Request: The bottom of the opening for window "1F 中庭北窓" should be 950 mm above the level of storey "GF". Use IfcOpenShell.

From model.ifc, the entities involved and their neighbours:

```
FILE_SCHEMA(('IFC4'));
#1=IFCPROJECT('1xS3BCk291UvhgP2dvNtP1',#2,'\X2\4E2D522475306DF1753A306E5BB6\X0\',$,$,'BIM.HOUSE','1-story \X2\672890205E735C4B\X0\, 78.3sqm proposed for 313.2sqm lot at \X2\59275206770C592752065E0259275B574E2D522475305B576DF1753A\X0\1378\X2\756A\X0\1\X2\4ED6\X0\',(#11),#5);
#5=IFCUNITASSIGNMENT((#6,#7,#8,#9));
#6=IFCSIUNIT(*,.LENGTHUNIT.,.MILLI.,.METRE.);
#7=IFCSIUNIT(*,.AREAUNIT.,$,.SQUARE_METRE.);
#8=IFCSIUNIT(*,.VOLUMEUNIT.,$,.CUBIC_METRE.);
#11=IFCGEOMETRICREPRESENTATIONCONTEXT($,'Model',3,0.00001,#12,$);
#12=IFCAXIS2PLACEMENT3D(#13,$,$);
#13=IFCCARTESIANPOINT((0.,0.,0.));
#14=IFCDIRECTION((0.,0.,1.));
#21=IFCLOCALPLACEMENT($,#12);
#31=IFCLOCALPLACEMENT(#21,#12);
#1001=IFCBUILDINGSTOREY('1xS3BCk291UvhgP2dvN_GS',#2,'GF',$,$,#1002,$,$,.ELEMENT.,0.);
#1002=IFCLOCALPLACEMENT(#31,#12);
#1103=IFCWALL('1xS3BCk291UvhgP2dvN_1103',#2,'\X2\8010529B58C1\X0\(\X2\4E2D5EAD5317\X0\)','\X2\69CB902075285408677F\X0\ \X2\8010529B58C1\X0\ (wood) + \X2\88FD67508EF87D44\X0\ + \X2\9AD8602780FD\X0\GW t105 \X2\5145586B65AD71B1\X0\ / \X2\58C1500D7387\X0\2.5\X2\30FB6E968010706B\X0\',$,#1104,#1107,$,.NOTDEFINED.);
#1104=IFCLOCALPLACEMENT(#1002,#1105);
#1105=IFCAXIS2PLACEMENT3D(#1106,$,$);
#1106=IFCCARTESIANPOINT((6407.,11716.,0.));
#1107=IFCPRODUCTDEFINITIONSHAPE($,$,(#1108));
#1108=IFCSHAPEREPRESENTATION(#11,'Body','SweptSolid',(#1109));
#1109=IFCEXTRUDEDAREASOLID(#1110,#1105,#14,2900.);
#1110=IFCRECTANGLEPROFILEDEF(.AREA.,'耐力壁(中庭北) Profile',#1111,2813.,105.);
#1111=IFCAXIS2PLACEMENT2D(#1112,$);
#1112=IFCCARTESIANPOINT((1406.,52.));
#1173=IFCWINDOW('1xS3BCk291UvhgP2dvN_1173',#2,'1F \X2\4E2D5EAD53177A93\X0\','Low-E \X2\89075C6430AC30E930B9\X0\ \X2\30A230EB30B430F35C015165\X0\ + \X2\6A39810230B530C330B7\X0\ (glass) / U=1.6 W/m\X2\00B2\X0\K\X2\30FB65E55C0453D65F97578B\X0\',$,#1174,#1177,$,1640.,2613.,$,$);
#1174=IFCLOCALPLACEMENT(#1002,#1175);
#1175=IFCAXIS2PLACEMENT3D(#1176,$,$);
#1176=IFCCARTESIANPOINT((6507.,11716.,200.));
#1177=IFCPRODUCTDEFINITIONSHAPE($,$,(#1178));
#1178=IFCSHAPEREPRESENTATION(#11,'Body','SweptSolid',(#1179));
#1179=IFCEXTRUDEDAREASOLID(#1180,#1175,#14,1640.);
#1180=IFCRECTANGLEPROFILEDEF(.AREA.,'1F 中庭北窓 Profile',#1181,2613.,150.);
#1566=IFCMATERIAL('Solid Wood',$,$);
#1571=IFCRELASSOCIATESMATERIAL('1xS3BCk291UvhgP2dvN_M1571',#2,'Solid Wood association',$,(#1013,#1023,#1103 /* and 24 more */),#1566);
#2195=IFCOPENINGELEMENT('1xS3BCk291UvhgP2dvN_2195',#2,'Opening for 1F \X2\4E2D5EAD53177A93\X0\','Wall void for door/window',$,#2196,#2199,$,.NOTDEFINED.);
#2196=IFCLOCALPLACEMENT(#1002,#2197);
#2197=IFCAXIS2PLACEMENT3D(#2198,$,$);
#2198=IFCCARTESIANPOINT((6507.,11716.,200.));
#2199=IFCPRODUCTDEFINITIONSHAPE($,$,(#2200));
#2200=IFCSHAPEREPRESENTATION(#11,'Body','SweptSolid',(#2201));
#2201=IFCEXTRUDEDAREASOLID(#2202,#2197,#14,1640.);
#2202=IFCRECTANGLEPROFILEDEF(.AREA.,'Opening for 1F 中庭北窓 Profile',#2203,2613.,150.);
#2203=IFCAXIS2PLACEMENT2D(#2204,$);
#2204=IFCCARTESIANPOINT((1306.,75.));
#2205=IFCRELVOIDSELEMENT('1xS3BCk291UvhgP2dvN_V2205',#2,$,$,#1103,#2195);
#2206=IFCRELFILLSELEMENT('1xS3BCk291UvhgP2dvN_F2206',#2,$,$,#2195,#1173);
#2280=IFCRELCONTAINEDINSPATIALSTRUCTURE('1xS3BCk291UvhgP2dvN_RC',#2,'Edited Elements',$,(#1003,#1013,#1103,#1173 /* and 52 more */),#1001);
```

```python
import numpy as np
import ifcopenshell
import ifcopenshell.api.geometry
import ifcopenshell.geom
import ifcopenshell.util.element
import ifcopenshell.util.placement
import ifcopenshell.util.shape
import ifcopenshell.util.unit

model = ifcopenshell.open("model.ifc")
unit_scale = ifcopenshell.util.unit.calculate_unit_scale(model)

window = model.by_id(1173)
opening = window.FillsVoids[0].RelatingOpeningElement
storey = ifcopenshell.util.element.get_container(window, ifc_class="IfcBuildingStorey")
level = ifcopenshell.util.placement.get_local_placement(storey.ObjectPlacement)[2, 3]

# The opening's origin need not be at the sill, so measure its lowest point.
shape = ifcopenshell.geom.create_shape(ifcopenshell.geom.settings(), opening)
bottom = ifcopenshell.util.shape.get_shape_bottom_elevation(shape, shape.geometry) / unit_scale
dz = level + 950.0 - bottom

shift = np.array([0.0, 0.0, dz])
# The window is not placed relative to its opening, so move both.
for product in (opening, window):
    matrix = ifcopenshell.util.placement.get_local_placement(product.ObjectPlacement)
    matrix[:3, 3] += shift
    ifcopenshell.api.geometry.edit_object_placement(model, product=product, matrix=matrix, is_si=False)

print(f"moved by {dz * unit_scale:+.3f} m")

model.write("model-out.ifc")
```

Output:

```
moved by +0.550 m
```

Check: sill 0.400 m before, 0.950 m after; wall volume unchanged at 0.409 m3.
